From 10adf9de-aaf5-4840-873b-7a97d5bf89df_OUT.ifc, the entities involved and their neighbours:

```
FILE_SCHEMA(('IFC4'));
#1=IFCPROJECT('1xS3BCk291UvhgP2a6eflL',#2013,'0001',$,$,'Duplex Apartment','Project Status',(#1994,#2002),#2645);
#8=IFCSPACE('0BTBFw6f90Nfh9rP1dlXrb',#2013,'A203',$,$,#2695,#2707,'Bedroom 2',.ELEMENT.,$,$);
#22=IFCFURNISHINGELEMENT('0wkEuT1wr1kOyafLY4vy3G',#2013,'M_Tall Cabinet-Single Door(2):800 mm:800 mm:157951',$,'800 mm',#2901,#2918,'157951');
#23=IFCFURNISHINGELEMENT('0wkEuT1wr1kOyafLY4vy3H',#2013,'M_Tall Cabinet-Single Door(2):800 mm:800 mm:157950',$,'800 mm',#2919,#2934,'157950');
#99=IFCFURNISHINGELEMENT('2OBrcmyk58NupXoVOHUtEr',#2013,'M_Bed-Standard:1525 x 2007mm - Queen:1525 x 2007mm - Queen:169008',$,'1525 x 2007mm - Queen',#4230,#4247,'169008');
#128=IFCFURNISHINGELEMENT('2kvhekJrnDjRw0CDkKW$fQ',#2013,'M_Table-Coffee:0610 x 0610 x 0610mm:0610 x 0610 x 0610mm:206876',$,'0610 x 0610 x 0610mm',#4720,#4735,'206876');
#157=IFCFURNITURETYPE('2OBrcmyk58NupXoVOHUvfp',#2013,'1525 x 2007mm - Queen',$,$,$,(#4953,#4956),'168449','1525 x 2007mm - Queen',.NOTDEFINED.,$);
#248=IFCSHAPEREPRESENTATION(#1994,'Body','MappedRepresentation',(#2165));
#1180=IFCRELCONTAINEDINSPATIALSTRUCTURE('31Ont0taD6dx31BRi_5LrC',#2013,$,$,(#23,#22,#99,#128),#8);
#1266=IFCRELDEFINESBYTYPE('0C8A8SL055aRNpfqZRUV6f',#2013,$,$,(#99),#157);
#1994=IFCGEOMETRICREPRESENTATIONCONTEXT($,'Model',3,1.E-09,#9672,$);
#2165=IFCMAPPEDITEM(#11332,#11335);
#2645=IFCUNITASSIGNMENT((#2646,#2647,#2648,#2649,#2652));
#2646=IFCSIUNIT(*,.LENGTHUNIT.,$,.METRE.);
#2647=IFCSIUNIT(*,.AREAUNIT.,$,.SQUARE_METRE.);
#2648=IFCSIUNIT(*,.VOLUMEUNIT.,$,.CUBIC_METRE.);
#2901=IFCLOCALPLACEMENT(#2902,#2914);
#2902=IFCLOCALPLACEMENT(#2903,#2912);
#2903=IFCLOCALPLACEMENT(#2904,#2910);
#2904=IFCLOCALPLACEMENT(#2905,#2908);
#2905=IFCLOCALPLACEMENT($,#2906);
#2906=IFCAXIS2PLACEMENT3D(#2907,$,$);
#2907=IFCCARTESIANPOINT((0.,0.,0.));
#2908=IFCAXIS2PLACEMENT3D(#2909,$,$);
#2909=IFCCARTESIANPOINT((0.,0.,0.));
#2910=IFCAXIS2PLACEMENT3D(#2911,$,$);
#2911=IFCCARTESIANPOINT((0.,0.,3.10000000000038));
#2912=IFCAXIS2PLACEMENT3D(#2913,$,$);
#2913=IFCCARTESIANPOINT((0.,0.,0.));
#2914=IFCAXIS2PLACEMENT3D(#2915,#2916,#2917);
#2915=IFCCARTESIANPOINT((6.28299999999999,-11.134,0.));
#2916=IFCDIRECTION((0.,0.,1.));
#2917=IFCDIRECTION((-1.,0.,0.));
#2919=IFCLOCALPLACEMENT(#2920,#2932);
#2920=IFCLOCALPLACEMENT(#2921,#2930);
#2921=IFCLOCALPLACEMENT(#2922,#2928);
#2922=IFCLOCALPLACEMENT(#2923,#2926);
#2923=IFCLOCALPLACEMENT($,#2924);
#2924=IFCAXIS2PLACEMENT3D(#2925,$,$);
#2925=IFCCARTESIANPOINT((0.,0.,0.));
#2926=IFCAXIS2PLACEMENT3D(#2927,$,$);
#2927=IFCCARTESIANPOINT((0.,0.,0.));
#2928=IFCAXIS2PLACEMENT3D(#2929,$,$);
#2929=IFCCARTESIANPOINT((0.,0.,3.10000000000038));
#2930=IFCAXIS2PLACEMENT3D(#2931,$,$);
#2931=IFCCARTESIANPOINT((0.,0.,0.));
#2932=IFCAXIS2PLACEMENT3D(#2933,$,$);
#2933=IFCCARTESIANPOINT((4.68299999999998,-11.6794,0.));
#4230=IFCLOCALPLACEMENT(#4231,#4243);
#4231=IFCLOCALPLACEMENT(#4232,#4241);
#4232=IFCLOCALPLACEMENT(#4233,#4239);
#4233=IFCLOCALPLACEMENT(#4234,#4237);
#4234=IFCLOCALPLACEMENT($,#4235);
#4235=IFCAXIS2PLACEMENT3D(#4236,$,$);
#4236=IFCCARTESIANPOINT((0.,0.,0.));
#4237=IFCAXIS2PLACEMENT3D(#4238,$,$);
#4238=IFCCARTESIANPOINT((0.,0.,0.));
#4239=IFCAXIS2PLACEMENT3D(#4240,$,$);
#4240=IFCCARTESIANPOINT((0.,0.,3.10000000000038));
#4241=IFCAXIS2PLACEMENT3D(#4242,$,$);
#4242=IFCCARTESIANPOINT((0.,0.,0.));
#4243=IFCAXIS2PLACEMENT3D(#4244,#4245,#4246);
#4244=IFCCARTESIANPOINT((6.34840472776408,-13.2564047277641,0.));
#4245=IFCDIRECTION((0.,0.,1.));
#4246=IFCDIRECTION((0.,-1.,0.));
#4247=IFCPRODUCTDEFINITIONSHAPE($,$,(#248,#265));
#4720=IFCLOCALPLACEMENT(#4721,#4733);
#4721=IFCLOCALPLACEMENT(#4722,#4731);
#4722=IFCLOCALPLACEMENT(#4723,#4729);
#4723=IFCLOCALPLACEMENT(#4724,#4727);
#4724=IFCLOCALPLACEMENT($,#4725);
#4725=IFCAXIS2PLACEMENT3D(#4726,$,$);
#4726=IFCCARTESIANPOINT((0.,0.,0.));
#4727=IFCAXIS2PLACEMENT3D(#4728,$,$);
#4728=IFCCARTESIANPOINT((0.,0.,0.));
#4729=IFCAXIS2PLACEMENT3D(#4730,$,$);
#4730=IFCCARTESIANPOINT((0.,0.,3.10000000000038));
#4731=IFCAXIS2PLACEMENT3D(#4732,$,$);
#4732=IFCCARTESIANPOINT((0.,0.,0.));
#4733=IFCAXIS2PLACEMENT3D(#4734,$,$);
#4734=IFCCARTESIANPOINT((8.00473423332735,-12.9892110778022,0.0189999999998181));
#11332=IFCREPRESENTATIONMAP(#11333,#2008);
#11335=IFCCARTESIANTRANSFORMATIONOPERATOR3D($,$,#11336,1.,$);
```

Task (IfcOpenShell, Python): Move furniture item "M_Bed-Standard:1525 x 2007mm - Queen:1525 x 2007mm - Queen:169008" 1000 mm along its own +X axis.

```python
import ifcopenshell
import ifcopenshell.api.geometry
import ifcopenshell.util.placement

model = ifcopenshell.open("10adf9de-aaf5-4840-873b-7a97d5bf89df_OUT.ifc")

item = model.by_guid("2OBrcmyk58NupXoVOHUtEr")
matrix = ifcopenshell.util.placement.get_local_placement(item.ObjectPlacement)
matrix[:3, 3] += matrix[:3, 0] * 1.0
ifcopenshell.api.geometry.edit_object_placement(model, product=item, matrix=matrix, is_si=False)

print(ifcopenshell.util.placement.get_local_placement(item.ObjectPlacement).round(3) + 0.0)

model.write("10adf9de-aaf5-4840-873b-7a97d5bf89df_OUT-out.ifc")
```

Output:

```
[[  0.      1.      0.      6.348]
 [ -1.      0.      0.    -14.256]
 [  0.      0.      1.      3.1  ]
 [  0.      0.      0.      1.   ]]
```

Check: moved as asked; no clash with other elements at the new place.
